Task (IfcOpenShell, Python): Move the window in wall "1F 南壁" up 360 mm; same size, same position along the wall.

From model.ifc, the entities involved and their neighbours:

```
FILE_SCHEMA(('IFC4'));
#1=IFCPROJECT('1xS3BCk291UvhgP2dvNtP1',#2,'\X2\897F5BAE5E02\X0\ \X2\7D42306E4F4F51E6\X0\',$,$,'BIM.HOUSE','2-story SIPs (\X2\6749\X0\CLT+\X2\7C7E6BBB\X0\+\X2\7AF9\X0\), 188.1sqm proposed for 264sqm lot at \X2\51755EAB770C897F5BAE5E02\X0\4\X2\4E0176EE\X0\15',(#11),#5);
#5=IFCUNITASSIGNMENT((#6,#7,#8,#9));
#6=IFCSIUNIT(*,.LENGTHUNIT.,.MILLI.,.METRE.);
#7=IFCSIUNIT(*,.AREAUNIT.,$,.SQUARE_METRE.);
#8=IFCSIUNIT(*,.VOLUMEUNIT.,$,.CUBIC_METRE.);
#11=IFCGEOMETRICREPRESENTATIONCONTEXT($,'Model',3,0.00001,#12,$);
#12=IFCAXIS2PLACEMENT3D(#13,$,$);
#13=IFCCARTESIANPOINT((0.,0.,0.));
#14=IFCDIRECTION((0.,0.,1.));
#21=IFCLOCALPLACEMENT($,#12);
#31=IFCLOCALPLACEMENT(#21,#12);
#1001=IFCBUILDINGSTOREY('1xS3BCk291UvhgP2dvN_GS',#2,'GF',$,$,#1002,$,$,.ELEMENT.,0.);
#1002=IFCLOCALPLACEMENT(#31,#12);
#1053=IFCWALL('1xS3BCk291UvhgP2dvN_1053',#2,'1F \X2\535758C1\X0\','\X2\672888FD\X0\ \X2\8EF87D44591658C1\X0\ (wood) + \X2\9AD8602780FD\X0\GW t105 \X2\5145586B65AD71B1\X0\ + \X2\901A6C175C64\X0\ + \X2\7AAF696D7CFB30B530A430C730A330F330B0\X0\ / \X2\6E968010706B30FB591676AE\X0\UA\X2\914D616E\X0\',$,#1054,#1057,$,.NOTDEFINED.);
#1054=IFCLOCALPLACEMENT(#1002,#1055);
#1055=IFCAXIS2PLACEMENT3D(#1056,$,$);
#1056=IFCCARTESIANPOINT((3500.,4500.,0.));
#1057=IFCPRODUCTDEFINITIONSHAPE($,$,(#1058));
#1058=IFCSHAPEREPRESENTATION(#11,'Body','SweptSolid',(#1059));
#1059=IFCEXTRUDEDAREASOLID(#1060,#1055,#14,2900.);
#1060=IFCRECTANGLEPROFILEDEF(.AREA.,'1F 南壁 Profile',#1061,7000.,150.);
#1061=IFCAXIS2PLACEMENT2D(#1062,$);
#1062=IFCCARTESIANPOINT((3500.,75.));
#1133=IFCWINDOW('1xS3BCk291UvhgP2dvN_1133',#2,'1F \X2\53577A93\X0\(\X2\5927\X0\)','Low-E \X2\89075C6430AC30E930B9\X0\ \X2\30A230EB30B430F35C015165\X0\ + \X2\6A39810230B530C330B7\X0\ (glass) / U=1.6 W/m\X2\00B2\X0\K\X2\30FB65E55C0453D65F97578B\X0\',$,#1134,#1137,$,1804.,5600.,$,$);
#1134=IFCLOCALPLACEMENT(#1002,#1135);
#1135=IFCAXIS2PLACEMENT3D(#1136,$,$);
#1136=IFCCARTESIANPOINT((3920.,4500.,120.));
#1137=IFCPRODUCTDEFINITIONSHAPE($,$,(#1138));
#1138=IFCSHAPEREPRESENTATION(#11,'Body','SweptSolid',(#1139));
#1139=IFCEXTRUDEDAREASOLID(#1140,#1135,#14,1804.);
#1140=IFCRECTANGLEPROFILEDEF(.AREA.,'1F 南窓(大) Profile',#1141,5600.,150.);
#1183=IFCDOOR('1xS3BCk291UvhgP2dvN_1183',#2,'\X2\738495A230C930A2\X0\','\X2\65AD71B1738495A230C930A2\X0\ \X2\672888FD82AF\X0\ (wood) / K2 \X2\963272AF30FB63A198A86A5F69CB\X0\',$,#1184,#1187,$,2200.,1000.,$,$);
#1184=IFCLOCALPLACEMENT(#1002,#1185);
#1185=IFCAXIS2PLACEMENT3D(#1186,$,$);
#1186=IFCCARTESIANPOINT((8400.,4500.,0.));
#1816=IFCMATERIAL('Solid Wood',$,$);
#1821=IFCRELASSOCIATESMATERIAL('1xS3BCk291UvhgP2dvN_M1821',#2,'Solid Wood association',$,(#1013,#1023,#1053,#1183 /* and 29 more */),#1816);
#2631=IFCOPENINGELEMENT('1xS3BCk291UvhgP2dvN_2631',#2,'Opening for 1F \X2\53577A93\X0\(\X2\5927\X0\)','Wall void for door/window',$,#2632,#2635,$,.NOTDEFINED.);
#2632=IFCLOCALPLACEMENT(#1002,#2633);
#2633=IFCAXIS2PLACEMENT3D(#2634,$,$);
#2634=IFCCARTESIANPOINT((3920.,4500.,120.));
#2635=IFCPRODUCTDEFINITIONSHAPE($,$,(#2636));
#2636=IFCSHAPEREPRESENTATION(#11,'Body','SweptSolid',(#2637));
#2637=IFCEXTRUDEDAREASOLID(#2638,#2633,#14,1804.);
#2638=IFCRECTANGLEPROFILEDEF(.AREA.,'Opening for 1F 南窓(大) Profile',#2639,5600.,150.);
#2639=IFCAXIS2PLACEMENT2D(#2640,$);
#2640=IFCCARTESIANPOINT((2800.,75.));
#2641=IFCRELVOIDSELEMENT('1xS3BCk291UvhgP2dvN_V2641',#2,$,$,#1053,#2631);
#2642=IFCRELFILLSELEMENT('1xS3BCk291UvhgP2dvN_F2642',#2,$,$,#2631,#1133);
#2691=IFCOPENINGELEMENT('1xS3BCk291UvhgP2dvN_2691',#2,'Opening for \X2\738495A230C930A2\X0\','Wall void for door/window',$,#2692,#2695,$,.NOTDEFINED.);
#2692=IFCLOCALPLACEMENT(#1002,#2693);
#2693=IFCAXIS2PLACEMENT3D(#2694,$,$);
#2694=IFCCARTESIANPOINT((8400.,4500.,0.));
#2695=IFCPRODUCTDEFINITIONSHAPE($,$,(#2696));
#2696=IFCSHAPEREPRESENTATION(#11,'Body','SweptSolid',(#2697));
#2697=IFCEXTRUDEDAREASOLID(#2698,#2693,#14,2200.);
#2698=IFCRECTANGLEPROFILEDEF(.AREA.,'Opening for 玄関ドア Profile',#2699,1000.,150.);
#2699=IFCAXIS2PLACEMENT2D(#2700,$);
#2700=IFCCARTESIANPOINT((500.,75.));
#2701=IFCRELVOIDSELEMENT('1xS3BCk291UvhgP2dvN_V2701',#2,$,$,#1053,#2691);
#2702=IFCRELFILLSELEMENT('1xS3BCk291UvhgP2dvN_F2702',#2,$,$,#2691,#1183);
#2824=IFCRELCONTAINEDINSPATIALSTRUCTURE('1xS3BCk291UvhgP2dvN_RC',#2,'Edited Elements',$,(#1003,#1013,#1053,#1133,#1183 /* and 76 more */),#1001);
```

```python
import numpy as np
import ifcopenshell
import ifcopenshell.api.geometry
import ifcopenshell.util.placement
import ifcopenshell.util.unit

model = ifcopenshell.open("model.ifc")
unit_scale = ifcopenshell.util.unit.calculate_unit_scale(model)

window = model.by_guid("1xS3BCk291UvhgP2dvN_1133")
opening = window.FillsVoids[0].RelatingOpeningElement
dz = 360.0

shift = np.array([0.0, 0.0, dz])
# The window is not placed relative to its opening, so move both.
for product in (opening, window):
    matrix = ifcopenshell.util.placement.get_local_placement(product.ObjectPlacement)
    matrix[:3, 3] += shift
    ifcopenshell.api.geometry.edit_object_placement(model, product=product, matrix=matrix, is_si=False)

print(f"moved by {dz * unit_scale:+.3f} m")

model.write("model_v2.ifc")
```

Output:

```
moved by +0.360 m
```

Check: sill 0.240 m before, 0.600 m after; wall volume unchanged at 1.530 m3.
